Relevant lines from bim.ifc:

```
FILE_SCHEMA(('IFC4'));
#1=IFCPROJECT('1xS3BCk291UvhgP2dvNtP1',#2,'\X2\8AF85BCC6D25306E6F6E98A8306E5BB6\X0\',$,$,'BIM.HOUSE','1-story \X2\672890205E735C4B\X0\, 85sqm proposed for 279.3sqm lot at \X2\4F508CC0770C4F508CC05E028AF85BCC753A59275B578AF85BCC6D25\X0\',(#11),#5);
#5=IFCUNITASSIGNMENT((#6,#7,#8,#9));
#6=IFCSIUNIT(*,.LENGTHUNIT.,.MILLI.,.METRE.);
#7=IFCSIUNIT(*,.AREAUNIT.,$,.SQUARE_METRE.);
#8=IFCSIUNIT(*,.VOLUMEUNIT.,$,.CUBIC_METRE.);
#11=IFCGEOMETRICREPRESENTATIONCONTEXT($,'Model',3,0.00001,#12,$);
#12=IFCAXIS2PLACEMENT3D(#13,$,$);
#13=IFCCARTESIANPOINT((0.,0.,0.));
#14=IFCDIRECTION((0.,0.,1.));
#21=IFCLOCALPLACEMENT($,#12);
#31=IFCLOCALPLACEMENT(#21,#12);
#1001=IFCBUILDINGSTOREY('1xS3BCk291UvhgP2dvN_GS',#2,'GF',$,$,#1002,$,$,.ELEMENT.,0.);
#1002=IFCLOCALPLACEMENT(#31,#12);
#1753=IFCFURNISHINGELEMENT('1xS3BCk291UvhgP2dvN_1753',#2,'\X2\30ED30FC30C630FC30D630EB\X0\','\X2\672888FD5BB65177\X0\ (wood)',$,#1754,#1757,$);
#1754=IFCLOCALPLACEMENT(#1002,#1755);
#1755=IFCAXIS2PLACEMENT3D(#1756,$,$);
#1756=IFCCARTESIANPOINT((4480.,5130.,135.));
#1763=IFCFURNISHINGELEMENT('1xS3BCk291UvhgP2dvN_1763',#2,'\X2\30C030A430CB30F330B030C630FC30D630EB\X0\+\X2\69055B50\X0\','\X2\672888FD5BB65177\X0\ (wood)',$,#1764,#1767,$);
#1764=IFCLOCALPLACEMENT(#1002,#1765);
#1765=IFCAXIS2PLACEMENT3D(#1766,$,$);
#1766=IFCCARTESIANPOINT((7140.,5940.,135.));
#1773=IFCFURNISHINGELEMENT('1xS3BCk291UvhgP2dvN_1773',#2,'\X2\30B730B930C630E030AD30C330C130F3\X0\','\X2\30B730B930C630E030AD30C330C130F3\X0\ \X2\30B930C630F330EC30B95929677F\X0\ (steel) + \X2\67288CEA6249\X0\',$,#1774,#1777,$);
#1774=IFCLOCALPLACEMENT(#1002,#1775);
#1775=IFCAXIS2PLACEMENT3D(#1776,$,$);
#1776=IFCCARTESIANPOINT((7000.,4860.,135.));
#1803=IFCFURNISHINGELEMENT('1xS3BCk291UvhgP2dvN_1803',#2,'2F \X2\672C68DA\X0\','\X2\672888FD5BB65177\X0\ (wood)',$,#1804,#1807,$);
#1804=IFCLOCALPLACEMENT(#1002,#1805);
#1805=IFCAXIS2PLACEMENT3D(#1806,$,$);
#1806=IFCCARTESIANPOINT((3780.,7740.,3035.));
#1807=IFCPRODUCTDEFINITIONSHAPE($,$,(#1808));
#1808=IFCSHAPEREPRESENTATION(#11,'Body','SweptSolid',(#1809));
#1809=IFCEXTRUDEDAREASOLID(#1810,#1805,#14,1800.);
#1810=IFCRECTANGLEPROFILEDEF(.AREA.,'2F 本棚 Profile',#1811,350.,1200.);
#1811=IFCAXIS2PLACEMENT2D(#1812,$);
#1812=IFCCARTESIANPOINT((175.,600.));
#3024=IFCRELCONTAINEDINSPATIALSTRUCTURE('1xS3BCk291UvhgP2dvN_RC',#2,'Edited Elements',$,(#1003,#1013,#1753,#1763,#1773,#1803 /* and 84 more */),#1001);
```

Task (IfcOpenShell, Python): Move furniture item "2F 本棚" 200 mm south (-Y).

```python
import ifcopenshell
import ifcopenshell.api.geometry
import ifcopenshell.util.placement
import ifcopenshell.util.unit

model = ifcopenshell.open("bim.ifc")
unit_scale = ifcopenshell.util.unit.calculate_unit_scale(model)

item = model.by_id(1803)
matrix = ifcopenshell.util.placement.get_local_placement(item.ObjectPlacement)
matrix[1, 3] -= 0.2 / unit_scale
ifcopenshell.api.geometry.edit_object_placement(model, product=item, matrix=matrix, is_si=False)

print(ifcopenshell.util.placement.get_local_placement(item.ObjectPlacement).round(3) + 0.0)

model.write("bim_v2.ifc")
```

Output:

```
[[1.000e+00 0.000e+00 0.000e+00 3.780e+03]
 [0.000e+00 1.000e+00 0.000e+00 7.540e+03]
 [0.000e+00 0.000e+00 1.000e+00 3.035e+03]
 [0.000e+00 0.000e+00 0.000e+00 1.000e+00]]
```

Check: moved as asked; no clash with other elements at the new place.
